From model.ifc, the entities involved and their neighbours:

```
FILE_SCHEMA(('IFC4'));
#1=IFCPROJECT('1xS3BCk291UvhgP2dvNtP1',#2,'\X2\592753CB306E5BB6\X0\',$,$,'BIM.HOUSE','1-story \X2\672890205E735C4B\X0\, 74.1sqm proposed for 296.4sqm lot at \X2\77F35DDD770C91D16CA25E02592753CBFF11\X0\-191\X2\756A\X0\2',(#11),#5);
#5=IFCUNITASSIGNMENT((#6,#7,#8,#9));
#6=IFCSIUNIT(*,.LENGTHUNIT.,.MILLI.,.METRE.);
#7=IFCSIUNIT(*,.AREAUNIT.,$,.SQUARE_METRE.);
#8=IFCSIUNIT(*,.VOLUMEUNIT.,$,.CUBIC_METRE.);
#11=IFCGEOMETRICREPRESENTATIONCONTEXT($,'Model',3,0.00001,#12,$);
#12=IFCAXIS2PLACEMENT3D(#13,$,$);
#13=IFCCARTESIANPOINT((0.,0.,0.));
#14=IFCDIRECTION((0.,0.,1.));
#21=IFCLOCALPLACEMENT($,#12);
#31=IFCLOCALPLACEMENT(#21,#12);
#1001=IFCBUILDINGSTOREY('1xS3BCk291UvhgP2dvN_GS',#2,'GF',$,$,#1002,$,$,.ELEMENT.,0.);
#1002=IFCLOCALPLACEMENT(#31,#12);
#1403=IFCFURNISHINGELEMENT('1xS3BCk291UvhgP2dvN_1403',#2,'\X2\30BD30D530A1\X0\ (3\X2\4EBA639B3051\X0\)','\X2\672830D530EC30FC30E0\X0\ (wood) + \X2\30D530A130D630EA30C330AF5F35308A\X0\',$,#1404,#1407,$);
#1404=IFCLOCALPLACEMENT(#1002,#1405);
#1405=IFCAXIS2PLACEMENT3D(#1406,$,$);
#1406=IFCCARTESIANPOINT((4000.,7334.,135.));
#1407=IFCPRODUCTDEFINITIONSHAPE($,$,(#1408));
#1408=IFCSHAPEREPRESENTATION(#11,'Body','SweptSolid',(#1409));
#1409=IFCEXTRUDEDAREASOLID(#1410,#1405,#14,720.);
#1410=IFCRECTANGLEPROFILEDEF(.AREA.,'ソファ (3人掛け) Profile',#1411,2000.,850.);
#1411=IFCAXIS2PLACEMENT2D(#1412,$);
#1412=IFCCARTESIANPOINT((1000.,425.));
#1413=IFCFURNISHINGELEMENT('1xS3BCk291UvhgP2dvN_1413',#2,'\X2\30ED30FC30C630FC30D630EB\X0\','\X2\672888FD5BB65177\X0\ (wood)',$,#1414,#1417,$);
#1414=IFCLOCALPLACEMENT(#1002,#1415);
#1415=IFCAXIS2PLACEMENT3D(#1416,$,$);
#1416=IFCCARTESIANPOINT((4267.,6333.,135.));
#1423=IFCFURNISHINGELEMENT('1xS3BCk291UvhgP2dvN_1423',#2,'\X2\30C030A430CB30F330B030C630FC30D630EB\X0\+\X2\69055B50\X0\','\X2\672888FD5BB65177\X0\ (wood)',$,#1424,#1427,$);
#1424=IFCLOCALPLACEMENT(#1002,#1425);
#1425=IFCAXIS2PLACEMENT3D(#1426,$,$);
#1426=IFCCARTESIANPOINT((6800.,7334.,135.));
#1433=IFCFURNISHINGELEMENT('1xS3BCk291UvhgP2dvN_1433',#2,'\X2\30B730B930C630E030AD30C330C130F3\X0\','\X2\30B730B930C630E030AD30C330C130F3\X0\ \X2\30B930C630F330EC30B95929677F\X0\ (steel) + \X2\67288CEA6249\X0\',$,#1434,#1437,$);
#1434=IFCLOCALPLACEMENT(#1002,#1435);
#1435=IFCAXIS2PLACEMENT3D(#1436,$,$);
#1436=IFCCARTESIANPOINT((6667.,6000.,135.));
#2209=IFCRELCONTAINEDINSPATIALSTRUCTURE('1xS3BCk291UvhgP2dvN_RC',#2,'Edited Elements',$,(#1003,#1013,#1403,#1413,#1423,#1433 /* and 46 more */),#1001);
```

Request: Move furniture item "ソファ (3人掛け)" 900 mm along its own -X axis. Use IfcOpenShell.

```python
import ifcopenshell
import ifcopenshell.api.geometry
import ifcopenshell.util.placement

model = ifcopenshell.open("model.ifc")

item = model.by_guid("1xS3BCk291UvhgP2dvN_1403")
matrix = ifcopenshell.util.placement.get_local_placement(item.ObjectPlacement)
matrix[:3, 3] -= matrix[:3, 0] * 900.0
ifcopenshell.api.geometry.edit_object_placement(model, product=item, matrix=matrix, is_si=False)

print(ifcopenshell.util.placement.get_local_placement(item.ObjectPlacement).round(3) + 0.0)

model.write("model-out.ifc")
```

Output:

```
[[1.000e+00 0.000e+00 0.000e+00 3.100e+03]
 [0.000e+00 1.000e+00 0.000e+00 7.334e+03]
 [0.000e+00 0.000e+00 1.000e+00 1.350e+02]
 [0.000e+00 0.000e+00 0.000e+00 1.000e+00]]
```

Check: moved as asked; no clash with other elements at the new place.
